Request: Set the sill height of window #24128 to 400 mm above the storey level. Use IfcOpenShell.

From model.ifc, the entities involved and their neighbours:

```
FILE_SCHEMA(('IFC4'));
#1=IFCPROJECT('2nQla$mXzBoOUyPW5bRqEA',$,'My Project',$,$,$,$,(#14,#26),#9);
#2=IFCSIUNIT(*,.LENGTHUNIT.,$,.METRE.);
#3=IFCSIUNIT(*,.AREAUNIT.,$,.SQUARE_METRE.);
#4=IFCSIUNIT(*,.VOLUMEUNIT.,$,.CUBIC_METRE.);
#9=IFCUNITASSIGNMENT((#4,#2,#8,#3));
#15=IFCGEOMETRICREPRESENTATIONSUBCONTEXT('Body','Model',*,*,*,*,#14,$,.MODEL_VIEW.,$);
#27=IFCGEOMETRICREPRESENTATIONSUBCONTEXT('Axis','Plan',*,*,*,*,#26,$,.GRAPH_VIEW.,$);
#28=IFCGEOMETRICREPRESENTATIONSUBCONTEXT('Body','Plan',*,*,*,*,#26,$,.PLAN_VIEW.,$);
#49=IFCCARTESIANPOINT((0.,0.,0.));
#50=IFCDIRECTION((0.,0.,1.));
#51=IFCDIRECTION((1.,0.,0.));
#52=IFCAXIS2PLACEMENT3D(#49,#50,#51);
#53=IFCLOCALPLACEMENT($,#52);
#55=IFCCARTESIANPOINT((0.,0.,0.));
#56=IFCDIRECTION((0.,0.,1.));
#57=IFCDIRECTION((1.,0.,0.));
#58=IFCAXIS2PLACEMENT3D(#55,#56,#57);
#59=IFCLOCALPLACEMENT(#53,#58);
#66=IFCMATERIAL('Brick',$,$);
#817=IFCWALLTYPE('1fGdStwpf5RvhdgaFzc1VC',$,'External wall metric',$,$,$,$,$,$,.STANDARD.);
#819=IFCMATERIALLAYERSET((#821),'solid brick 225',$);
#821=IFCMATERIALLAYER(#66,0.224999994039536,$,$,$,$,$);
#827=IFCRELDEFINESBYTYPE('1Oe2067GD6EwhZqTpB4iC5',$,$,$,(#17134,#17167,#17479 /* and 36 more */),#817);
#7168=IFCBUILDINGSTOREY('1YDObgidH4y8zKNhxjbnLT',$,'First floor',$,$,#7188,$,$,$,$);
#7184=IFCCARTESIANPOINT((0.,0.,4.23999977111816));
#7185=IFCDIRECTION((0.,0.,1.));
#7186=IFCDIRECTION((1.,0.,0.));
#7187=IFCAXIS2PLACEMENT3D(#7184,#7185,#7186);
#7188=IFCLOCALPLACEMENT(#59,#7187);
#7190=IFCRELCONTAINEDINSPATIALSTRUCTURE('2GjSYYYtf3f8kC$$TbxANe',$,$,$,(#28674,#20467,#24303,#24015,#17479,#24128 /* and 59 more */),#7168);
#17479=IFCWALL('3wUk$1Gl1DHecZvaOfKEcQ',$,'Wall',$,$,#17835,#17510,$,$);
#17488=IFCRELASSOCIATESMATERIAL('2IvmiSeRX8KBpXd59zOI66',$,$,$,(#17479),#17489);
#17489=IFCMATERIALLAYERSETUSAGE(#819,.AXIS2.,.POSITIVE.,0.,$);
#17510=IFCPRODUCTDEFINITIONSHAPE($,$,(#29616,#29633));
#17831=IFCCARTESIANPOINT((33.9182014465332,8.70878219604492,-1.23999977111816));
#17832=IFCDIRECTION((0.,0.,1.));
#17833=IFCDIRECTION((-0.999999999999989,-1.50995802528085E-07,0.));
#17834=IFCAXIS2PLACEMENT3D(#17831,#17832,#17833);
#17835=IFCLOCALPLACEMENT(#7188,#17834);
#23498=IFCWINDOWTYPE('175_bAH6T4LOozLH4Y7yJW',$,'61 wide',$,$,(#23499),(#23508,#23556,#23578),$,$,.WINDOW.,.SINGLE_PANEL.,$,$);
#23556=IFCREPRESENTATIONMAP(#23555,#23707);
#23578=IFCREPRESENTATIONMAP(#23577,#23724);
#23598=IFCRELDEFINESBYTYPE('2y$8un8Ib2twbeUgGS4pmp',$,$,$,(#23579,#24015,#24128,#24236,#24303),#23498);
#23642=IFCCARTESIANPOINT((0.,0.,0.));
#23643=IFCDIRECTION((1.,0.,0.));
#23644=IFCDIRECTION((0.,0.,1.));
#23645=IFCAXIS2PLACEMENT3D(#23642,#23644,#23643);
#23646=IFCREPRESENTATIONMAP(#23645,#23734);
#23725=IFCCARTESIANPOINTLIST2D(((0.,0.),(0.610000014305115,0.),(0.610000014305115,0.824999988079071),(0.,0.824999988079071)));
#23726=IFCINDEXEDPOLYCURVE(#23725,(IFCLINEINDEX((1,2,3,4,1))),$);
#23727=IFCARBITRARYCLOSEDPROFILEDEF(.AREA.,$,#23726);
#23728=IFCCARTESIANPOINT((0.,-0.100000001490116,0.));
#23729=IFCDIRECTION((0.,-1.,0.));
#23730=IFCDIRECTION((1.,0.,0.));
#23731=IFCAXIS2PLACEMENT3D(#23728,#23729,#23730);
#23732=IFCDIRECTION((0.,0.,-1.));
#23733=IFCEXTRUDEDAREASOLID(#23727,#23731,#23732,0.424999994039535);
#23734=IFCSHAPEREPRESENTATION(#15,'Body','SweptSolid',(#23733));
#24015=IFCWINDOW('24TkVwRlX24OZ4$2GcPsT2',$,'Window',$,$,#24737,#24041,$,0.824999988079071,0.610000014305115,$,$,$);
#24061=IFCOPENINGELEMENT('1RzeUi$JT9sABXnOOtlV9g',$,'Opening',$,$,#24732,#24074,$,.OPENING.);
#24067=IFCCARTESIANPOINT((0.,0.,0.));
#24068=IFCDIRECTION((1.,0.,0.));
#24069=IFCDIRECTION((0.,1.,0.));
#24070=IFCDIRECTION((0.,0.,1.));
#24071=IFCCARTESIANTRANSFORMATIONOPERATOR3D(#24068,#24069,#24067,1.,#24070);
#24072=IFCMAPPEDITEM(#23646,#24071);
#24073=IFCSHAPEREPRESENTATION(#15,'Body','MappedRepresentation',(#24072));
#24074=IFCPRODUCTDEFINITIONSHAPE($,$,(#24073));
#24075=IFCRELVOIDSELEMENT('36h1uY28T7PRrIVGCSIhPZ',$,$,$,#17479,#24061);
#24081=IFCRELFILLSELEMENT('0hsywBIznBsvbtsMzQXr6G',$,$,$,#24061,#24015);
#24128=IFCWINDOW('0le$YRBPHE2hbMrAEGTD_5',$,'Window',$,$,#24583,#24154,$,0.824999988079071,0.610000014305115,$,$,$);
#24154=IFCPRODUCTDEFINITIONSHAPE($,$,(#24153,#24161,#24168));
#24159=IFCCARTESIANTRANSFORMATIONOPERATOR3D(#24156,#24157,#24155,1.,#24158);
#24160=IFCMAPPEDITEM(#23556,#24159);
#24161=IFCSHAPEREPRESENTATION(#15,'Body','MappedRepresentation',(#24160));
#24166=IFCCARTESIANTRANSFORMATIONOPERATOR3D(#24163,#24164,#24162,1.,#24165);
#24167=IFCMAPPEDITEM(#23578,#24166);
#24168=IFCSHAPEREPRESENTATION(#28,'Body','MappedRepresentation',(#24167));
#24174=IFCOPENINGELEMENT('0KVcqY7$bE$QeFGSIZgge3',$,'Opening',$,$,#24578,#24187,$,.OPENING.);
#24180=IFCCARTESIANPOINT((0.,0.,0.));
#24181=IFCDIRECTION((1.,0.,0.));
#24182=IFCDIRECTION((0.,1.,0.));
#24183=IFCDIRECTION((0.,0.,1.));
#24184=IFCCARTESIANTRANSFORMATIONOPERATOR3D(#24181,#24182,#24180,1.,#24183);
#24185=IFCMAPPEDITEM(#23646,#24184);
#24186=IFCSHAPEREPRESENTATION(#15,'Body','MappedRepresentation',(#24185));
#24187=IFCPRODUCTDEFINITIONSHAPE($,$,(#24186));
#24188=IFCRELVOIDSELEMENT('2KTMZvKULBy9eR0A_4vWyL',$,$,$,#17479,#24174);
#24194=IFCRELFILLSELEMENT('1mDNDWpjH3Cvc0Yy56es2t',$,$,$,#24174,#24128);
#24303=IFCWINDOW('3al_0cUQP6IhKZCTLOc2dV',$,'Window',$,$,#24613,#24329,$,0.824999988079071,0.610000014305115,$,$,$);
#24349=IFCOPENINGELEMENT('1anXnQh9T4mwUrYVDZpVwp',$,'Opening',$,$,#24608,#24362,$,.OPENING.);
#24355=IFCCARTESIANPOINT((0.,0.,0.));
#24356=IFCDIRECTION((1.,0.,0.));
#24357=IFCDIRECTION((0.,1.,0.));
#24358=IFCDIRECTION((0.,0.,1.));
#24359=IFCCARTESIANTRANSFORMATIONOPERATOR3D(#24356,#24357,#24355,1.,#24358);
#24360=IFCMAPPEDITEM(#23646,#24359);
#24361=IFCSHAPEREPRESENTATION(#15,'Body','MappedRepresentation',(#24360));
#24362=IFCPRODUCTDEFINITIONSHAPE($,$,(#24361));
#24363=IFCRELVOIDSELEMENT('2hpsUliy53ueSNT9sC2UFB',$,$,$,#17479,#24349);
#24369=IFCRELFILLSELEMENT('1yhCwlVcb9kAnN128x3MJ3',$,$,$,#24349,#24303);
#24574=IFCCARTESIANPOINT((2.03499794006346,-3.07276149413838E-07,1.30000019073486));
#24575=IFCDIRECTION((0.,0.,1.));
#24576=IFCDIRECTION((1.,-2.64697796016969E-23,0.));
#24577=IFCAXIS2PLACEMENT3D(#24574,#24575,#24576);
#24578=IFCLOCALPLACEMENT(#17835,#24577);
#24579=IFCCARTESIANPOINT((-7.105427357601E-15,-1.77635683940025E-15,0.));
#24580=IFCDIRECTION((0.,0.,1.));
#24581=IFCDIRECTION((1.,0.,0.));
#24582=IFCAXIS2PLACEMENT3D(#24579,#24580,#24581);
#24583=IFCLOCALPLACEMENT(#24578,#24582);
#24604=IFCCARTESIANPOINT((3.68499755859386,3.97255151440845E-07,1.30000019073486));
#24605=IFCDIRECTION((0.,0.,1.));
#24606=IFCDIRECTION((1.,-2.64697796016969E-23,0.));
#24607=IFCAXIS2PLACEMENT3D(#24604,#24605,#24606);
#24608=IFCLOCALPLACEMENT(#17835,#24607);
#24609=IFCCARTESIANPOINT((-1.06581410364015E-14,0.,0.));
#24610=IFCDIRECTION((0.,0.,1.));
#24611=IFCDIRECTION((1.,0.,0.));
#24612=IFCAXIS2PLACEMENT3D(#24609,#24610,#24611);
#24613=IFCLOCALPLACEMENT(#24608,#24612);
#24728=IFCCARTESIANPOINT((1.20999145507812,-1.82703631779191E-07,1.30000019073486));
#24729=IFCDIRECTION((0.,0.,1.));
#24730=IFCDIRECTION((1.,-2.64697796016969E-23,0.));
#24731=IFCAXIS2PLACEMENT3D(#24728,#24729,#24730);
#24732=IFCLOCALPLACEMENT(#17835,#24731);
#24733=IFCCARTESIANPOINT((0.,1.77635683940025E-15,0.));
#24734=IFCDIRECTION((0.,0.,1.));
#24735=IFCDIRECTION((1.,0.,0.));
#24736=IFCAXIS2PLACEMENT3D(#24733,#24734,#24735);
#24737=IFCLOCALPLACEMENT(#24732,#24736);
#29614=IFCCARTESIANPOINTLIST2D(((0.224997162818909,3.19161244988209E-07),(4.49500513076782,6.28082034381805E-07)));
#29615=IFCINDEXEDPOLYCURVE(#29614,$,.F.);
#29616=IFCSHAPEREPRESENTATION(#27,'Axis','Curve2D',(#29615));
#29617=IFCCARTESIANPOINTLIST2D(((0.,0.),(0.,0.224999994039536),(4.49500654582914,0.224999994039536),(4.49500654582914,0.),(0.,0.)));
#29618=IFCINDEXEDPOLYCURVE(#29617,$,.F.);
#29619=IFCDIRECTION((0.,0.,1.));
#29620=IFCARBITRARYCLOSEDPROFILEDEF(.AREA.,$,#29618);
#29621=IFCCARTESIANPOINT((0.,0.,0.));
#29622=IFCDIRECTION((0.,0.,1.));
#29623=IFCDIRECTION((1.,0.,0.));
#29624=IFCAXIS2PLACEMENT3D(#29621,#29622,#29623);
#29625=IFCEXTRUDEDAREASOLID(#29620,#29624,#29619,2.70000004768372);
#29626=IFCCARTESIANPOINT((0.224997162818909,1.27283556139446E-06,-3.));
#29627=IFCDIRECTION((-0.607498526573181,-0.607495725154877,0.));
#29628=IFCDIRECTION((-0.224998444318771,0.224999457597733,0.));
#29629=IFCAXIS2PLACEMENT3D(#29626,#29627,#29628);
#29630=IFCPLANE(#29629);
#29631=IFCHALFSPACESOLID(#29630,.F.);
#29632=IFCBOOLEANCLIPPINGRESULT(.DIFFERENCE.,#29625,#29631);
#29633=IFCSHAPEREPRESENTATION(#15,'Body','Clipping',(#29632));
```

```python
import numpy as np
import ifcopenshell
import ifcopenshell.api.geometry
import ifcopenshell.geom
import ifcopenshell.util.element
import ifcopenshell.util.placement
import ifcopenshell.util.shape
import ifcopenshell.util.unit

model = ifcopenshell.open("model.ifc")
unit_scale = ifcopenshell.util.unit.calculate_unit_scale(model)

window = model.by_id(24128)
opening = window.FillsVoids[0].RelatingOpeningElement
storey = ifcopenshell.util.element.get_container(window, ifc_class="IfcBuildingStorey")
level = ifcopenshell.util.placement.get_local_placement(storey.ObjectPlacement)[2, 3]

# The opening's origin need not be at the sill, so measure its lowest point.
shape = ifcopenshell.geom.create_shape(ifcopenshell.geom.settings(), opening)
bottom = ifcopenshell.util.shape.get_shape_bottom_elevation(shape, shape.geometry) / unit_scale
dz = level + 0.4 / unit_scale - bottom

shift = np.array([0.0, 0.0, dz])
# The window is placed relative to its opening, so it follows when the opening moves.
matrix = ifcopenshell.util.placement.get_local_placement(opening.ObjectPlacement)
matrix[:3, 3] += shift
ifcopenshell.api.geometry.edit_object_placement(
    model, product=opening, matrix=matrix, is_si=False, should_transform_children=True
)

print(f"moved by {dz * unit_scale:+.3f} m")

model.write("model_edited.ifc")
```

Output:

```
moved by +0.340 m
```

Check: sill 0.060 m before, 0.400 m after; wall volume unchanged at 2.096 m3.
